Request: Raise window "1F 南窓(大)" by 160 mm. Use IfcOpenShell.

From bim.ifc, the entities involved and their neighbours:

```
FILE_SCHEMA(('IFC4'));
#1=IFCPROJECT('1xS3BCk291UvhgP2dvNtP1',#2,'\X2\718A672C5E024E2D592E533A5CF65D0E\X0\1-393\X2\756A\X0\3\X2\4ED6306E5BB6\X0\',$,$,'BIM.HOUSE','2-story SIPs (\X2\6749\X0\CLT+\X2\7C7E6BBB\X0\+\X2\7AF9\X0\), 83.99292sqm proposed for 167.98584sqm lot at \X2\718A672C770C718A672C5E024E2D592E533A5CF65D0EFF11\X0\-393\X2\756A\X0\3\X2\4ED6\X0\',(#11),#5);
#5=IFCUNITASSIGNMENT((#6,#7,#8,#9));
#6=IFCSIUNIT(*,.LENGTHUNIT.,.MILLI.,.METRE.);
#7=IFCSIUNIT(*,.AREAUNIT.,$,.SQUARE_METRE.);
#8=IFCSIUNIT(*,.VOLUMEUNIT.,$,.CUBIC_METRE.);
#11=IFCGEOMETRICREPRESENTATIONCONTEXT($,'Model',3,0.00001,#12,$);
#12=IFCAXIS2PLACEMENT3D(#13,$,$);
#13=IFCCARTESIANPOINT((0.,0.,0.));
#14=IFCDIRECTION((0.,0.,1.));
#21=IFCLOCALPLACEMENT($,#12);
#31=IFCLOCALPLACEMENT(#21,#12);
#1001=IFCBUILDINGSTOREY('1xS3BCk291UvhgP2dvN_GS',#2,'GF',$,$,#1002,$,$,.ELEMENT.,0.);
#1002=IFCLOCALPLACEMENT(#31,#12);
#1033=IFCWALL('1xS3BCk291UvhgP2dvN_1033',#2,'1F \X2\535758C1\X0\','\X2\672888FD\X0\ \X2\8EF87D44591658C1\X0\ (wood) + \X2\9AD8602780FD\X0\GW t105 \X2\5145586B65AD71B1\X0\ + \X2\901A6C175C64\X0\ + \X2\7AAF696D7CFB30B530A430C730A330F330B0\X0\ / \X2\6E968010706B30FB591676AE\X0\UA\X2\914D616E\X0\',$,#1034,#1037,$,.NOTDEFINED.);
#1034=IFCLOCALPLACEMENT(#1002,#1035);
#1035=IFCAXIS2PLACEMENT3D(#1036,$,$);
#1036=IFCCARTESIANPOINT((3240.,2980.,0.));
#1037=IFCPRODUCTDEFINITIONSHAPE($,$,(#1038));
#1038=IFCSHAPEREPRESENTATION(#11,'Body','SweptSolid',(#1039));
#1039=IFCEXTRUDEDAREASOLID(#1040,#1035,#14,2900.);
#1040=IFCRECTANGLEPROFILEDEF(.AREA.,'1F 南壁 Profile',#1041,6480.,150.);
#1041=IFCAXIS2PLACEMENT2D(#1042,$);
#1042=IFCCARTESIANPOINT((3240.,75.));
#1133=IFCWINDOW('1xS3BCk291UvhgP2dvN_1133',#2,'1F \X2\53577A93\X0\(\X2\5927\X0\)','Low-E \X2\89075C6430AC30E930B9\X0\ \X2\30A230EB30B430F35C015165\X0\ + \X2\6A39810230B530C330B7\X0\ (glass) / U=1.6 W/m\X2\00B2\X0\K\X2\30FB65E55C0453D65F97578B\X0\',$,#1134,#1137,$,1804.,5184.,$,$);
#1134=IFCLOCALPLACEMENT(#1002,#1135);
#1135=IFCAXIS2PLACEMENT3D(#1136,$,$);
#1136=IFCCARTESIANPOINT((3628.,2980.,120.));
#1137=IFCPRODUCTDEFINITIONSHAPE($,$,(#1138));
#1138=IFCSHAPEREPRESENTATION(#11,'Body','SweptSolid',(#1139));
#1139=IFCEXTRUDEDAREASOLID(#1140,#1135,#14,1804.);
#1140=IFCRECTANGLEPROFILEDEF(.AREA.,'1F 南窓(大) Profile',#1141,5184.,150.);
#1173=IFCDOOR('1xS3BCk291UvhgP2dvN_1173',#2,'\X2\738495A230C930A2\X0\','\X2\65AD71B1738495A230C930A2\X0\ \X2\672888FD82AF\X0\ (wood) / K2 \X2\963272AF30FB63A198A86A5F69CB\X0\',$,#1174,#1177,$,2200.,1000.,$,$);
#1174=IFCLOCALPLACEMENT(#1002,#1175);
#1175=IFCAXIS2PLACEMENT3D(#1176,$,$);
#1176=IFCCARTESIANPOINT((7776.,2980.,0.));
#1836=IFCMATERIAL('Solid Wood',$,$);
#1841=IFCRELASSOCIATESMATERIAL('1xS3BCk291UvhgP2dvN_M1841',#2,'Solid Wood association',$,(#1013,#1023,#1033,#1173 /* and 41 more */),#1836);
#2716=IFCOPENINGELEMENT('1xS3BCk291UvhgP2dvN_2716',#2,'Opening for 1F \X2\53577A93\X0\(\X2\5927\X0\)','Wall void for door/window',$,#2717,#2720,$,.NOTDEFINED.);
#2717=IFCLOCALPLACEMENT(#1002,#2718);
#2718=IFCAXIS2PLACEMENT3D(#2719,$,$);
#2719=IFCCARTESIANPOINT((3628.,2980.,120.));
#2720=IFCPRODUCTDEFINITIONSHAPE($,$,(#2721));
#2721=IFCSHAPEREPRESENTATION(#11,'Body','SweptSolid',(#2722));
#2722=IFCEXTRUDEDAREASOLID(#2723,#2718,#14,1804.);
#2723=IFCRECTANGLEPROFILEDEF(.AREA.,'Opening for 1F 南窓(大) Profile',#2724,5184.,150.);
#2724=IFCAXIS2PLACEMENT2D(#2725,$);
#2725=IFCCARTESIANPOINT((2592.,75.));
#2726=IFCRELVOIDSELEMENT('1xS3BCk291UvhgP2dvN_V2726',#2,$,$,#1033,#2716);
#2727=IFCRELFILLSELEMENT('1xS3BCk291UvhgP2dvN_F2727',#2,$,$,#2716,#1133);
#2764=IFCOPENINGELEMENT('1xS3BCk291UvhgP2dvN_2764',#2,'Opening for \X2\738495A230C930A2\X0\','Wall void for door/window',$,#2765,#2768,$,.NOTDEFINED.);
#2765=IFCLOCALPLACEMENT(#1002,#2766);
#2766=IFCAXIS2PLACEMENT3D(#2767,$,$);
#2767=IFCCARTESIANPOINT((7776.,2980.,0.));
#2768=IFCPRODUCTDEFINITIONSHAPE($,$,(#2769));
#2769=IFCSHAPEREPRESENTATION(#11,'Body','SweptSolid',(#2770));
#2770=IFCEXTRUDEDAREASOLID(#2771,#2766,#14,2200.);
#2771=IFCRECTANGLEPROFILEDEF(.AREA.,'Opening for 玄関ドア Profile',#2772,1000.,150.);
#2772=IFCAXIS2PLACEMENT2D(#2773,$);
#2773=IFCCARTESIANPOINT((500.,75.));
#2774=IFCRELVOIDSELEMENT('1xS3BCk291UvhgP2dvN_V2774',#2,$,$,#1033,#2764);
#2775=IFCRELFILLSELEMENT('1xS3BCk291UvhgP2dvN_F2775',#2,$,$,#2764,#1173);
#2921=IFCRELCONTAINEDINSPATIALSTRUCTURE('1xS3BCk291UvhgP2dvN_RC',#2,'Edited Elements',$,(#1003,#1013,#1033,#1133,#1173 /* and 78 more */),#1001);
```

```python
import numpy as np
import ifcopenshell
import ifcopenshell.api.geometry
import ifcopenshell.util.placement
import ifcopenshell.util.unit

model = ifcopenshell.open("bim.ifc")
unit_scale = ifcopenshell.util.unit.calculate_unit_scale(model)

window = model.by_id(1133)
opening = window.FillsVoids[0].RelatingOpeningElement
dz = 160.0

shift = np.array([0.0, 0.0, dz])
# The window is not placed relative to its opening, so move both.
for product in (opening, window):
    matrix = ifcopenshell.util.placement.get_local_placement(product.ObjectPlacement)
    matrix[:3, 3] += shift
    ifcopenshell.api.geometry.edit_object_placement(model, product=product, matrix=matrix, is_si=False)

print(f"moved by {dz * unit_scale:+.3f} m")

model.write("bim_rev.ifc")
```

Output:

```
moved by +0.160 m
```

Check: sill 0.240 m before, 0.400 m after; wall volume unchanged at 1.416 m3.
